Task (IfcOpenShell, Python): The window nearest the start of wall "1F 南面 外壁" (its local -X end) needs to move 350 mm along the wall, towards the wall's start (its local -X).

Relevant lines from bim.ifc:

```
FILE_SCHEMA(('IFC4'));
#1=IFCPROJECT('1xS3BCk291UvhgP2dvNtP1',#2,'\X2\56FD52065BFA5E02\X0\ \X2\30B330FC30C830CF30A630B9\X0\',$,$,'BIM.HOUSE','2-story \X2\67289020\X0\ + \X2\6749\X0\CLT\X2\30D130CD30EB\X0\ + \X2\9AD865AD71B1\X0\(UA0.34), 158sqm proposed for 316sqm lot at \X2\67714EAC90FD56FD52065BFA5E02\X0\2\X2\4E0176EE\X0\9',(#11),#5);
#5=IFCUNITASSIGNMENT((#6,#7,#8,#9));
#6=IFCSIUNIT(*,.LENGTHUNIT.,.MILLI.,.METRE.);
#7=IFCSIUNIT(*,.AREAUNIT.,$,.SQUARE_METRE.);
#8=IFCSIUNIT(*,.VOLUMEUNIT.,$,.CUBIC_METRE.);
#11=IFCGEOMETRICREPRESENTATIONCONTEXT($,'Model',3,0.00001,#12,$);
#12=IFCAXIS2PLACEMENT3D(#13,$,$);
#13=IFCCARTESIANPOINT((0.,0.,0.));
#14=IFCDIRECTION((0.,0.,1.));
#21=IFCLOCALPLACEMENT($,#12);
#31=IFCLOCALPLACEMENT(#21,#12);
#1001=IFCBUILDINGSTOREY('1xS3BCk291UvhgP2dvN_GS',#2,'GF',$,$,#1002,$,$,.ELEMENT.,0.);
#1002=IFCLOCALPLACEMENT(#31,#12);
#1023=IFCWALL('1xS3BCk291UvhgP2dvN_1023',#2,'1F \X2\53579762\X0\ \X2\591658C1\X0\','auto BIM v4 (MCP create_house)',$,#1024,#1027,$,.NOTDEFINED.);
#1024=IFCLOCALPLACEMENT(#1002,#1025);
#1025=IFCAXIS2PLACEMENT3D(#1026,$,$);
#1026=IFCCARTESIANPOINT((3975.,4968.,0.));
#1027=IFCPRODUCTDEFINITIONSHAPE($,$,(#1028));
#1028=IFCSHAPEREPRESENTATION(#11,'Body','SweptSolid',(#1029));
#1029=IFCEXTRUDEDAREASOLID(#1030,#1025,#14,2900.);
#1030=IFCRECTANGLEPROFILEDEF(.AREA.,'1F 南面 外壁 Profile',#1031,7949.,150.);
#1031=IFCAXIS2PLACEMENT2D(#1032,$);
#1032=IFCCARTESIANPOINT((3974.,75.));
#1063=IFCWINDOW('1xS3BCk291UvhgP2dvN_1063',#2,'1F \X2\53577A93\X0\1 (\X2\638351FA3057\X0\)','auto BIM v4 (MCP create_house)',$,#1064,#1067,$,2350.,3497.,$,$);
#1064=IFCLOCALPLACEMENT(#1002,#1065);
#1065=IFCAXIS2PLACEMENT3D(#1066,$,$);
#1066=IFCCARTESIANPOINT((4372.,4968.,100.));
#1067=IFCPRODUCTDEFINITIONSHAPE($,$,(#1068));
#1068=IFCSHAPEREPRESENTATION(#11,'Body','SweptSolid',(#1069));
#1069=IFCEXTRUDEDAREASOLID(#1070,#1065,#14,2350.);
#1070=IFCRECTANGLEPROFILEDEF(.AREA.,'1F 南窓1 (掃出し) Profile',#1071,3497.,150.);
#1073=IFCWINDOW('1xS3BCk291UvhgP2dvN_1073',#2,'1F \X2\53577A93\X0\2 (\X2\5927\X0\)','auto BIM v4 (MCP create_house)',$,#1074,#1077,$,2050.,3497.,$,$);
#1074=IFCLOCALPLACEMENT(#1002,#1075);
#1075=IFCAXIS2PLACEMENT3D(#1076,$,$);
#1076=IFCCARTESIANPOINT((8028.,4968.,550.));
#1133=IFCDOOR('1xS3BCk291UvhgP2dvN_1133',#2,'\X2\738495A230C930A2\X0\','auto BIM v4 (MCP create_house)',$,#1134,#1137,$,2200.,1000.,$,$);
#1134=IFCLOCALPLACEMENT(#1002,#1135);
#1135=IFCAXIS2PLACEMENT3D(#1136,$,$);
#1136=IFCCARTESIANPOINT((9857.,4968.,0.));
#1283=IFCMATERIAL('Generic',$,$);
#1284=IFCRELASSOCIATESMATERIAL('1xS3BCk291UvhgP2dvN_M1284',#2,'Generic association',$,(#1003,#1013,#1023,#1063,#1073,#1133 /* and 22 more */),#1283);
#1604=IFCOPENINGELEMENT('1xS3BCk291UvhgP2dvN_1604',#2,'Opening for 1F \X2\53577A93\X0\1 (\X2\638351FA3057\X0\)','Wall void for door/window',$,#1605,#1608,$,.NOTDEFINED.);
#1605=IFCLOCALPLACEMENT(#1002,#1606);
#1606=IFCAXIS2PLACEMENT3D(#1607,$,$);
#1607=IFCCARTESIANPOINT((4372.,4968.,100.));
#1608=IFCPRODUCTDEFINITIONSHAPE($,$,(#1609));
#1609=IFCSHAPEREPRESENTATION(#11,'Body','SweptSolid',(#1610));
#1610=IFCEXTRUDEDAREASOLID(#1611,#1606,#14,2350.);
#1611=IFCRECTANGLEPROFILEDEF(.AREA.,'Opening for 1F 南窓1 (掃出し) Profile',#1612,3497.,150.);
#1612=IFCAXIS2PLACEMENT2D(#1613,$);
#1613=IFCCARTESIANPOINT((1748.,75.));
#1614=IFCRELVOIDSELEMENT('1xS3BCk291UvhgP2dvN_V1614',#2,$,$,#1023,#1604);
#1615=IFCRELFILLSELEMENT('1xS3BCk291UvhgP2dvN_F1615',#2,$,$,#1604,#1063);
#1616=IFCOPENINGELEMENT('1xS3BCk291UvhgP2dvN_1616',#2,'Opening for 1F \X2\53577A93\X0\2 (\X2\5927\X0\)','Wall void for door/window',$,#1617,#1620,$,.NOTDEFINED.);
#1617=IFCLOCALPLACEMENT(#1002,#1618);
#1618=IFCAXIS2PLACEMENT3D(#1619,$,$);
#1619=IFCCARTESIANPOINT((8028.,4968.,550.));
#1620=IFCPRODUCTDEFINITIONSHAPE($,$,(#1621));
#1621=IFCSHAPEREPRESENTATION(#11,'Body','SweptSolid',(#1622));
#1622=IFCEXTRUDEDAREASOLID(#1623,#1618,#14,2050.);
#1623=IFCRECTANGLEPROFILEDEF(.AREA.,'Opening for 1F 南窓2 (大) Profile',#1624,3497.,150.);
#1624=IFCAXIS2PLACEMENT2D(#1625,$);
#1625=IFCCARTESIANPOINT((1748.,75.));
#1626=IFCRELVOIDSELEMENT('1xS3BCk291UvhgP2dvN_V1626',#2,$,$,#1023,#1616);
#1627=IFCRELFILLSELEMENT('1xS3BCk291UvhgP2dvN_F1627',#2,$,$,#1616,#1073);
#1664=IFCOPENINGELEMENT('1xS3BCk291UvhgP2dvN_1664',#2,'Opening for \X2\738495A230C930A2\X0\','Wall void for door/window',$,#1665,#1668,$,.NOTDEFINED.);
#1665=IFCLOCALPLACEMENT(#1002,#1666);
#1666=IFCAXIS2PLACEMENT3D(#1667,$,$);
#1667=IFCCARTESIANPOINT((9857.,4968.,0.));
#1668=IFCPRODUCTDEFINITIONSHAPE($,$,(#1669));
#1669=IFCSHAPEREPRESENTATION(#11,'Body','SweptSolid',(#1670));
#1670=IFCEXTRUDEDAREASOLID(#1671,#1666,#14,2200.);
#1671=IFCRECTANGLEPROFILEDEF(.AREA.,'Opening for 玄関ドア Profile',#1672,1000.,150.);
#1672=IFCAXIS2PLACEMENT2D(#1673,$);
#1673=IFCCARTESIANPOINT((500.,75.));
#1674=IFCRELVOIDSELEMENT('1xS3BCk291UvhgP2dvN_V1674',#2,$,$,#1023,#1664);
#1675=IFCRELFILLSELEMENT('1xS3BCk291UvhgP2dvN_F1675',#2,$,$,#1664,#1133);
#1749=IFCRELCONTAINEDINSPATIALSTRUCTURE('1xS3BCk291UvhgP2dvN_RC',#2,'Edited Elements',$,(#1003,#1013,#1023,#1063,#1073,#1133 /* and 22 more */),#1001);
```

```python
import ifcopenshell
import ifcopenshell.api.geometry
import ifcopenshell.util.placement
import ifcopenshell.util.unit

model = ifcopenshell.open("bim.ifc")
unit_scale = ifcopenshell.util.unit.calculate_unit_scale(model)

window = model.by_guid("1xS3BCk291UvhgP2dvN_1063")
opening = window.FillsVoids[0].RelatingOpeningElement
wall = opening.VoidsElements[0].RelatingBuildingElement

wall_matrix = ifcopenshell.util.placement.get_local_placement(wall.ObjectPlacement)
shift = wall_matrix[:3, 0] * -0.35 / unit_scale
before = ifcopenshell.util.placement.get_local_placement(window.ObjectPlacement)[:3, 3].copy()

# The window is not placed relative to its opening, so move both.
for product in (opening, window):
    matrix = ifcopenshell.util.placement.get_local_placement(product.ObjectPlacement)
    matrix[:3, 3] += shift
    ifcopenshell.api.geometry.edit_object_placement(model, product=product, matrix=matrix, is_si=False)

after = ifcopenshell.util.placement.get_local_placement(window.ObjectPlacement)[:3, 3]
print("window moved by", (after - before).round(3) + 0.0)

model.write("bim_v2.ifc")
```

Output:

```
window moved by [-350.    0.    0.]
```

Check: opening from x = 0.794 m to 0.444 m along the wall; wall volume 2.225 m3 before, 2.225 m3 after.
